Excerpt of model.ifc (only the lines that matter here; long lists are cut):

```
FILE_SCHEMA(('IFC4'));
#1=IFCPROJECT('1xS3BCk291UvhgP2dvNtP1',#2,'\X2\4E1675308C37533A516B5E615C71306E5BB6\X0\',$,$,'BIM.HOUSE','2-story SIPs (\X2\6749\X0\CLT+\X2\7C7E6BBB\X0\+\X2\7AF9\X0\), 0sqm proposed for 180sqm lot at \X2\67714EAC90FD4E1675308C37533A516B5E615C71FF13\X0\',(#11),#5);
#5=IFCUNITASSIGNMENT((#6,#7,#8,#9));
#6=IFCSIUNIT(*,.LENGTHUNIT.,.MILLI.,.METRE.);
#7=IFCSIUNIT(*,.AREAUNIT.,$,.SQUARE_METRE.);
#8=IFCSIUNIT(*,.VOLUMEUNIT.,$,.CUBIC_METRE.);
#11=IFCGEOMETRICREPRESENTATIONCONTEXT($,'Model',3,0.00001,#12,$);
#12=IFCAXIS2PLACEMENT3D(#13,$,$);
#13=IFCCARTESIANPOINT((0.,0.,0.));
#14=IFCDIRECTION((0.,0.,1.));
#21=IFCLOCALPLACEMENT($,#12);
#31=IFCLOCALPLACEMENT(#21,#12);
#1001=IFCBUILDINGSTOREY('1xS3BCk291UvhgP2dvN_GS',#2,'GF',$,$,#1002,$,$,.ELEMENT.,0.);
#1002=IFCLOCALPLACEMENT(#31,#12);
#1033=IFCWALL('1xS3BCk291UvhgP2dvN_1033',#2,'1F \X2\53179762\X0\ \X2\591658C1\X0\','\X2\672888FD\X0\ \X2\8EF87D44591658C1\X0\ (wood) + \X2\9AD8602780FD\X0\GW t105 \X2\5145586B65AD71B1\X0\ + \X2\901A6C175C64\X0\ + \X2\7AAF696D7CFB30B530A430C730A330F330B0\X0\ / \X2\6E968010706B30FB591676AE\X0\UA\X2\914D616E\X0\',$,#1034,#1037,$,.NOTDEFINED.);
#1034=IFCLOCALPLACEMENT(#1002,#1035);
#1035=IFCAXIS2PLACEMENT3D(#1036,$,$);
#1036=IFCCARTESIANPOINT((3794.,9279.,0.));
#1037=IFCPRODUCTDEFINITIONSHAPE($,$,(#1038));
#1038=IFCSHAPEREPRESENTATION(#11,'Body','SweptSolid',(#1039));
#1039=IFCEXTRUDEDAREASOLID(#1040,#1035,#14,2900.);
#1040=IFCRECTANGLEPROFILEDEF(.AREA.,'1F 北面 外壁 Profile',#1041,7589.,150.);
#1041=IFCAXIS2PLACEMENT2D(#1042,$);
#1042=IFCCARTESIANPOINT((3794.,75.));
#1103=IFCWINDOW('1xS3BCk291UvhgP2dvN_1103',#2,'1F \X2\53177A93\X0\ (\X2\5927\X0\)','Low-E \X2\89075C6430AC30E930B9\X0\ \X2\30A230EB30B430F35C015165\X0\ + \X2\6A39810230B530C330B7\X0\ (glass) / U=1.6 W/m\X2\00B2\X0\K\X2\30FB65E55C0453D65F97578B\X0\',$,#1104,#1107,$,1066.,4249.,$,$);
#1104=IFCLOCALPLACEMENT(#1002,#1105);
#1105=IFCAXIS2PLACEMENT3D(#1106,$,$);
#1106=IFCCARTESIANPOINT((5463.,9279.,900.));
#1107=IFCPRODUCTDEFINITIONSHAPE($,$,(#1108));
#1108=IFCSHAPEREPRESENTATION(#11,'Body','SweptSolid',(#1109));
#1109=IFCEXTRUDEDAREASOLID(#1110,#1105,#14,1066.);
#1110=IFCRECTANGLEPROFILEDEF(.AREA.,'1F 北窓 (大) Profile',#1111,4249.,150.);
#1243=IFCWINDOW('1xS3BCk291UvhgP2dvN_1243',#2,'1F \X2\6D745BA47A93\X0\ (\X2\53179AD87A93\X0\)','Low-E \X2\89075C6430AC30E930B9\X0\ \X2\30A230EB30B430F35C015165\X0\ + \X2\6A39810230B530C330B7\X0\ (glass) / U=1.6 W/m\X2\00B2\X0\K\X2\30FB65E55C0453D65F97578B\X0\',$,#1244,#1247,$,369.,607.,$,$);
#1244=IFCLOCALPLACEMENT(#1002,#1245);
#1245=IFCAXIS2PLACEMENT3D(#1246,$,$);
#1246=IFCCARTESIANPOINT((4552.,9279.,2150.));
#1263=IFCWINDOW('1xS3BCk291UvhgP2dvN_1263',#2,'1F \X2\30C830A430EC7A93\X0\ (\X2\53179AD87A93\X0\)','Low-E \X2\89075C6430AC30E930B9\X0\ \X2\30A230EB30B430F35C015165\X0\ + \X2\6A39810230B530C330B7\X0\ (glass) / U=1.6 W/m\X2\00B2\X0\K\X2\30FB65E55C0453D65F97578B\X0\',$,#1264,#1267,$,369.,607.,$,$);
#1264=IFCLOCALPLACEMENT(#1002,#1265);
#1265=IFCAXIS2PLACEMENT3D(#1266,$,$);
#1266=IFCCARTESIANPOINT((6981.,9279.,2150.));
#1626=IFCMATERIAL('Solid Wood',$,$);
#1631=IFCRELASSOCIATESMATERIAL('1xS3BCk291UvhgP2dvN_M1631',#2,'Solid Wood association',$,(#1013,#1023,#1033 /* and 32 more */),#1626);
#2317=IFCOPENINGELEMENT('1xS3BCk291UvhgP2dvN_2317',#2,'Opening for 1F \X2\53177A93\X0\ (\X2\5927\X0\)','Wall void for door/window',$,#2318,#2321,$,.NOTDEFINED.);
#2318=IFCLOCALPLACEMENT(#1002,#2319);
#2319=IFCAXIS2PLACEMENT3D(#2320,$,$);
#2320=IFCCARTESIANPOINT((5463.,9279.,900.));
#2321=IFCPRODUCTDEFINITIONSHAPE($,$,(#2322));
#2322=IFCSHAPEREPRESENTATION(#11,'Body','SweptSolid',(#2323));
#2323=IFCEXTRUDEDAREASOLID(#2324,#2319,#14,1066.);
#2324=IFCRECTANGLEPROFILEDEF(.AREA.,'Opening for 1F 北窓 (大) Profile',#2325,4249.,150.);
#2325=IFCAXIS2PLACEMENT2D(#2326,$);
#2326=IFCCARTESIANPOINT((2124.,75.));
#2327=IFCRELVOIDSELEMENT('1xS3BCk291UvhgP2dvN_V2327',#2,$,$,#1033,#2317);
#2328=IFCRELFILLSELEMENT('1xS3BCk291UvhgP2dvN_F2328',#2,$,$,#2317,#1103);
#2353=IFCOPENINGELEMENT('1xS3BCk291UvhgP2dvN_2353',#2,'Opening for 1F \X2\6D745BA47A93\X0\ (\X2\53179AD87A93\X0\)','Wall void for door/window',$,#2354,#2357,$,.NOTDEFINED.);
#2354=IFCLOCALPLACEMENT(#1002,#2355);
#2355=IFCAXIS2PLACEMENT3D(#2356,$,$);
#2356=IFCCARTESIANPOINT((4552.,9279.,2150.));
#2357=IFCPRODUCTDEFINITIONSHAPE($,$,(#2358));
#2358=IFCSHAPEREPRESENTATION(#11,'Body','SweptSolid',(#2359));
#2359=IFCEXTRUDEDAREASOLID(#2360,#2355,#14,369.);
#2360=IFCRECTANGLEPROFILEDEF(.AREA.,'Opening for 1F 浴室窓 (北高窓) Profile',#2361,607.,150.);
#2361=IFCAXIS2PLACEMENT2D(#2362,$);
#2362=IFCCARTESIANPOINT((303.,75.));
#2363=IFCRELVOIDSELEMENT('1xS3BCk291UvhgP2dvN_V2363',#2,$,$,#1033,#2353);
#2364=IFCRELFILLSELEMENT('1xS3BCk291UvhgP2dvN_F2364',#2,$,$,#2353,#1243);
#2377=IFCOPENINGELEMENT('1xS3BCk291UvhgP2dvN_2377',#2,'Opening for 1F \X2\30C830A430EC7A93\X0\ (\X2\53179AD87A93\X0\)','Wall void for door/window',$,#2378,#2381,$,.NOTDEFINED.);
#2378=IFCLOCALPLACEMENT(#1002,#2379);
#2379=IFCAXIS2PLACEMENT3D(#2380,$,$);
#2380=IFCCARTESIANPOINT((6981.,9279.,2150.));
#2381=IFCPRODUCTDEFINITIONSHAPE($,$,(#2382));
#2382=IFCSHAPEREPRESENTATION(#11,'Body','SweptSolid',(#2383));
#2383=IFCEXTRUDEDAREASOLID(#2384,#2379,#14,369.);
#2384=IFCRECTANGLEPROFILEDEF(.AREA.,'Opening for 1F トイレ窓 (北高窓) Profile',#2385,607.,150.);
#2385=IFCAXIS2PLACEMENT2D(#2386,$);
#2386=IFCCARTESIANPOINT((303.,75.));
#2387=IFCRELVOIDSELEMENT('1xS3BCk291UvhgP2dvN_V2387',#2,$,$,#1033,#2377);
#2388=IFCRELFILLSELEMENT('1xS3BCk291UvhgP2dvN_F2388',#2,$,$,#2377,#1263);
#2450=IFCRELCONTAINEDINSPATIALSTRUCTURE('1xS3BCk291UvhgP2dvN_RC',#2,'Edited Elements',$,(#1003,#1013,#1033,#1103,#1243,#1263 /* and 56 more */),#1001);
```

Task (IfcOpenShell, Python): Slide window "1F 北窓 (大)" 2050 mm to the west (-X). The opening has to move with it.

```python
import ifcopenshell
import ifcopenshell.api.geometry
import ifcopenshell.util.placement
import ifcopenshell.util.unit

model = ifcopenshell.open("model.ifc")
unit_scale = ifcopenshell.util.unit.calculate_unit_scale(model)

window = model.by_guid("1xS3BCk291UvhgP2dvN_1103")
opening = window.FillsVoids[0].RelatingOpeningElement
wall = opening.VoidsElements[0].RelatingBuildingElement

wall_matrix = ifcopenshell.util.placement.get_local_placement(wall.ObjectPlacement)
shift = wall_matrix[:3, 0] * -2.05 / unit_scale
before = ifcopenshell.util.placement.get_local_placement(window.ObjectPlacement)[:3, 3].copy()

# The window is not placed relative to its opening, so move both.
for product in (opening, window):
    matrix = ifcopenshell.util.placement.get_local_placement(product.ObjectPlacement)
    matrix[:3, 3] += shift
    ifcopenshell.api.geometry.edit_object_placement(model, product=product, matrix=matrix, is_si=False)

after = ifcopenshell.util.placement.get_local_placement(window.ObjectPlacement)[:3, 3]
print("window moved by", (after - before).round(3) + 0.0)

model.write("model_rev.ifc")
```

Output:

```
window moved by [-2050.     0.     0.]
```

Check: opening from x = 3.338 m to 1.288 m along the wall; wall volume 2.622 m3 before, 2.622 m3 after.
